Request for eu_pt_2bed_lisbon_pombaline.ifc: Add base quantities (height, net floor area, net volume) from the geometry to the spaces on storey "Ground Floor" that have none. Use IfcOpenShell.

First a look at what the model holds.

```python
import ifcopenshell
import ifcopenshell.util.element
import ifcopenshell.util.unit

model = ifcopenshell.open("eu_pt_2bed_lisbon_pombaline.ifc")
print(model.schema)
for unit_type in ("LENGTHUNIT", "AREAUNIT", "VOLUMEUNIT"):
    print(unit_type, ifcopenshell.util.unit.calculate_unit_scale(model, unit_type))
storey = next(s for s in model.by_type("IfcBuildingStorey") if s.Name == "Ground Floor")
spaces = [e for e in ifcopenshell.util.element.get_decomposition(storey) if e.is_a("IfcSpace")]
for e in sorted(spaces, key=lambda e: e.id()):
    print(e.id(), e.is_a(), e.Name, list(ifcopenshell.util.element.get_psets(e, qtos_only=True)), sep=" | ")
```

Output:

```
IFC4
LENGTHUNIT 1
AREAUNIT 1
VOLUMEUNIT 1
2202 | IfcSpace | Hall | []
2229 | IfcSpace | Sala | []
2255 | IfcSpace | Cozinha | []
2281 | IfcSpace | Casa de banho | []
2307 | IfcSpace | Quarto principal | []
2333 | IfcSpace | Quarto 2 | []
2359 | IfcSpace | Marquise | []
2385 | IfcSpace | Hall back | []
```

```python
import ifcopenshell
import ifcopenshell.api.pset
import ifcopenshell.geom
import ifcopenshell.util.element
import ifcopenshell.util.shape
import ifcopenshell.util.unit

model = ifcopenshell.open("eu_pt_2bed_lisbon_pombaline.ifc")
unit_scale = ifcopenshell.util.unit.calculate_unit_scale(model)
area_scale = ifcopenshell.util.unit.calculate_unit_scale(model, "AREAUNIT")
volume_scale = ifcopenshell.util.unit.calculate_unit_scale(model, "VOLUMEUNIT")
settings = ifcopenshell.geom.settings()

storey = next(s for s in model.by_type("IfcBuildingStorey") if s.Name == "Ground Floor")
spaces = [e for e in ifcopenshell.util.element.get_decomposition(storey) if e.is_a("IfcSpace")]

for e in sorted(spaces, key=lambda e: e.id()):
    if ifcopenshell.util.element.get_psets(e, qtos_only=True, should_inherit=False):
        continue
    # Geometry comes back in metres, in the element's own axes.
    shape = ifcopenshell.geom.create_shape(settings, e)
    values = {
        "Height": ifcopenshell.util.shape.get_z(shape.geometry) / unit_scale,
        "NetFloorArea": ifcopenshell.util.shape.get_footprint_area(shape.geometry) / area_scale,
        "NetVolume": ifcopenshell.util.shape.get_volume(shape.geometry) / volume_scale,
    }
    qto = ifcopenshell.api.pset.add_qto(model, product=e, name="Qto_SpaceBaseQuantities")
    ifcopenshell.api.pset.edit_qto(model, qto=qto, properties=values)
    print(e.id(), {k: round(v, 3) for k, v in values.items()})

model.write("eu_pt_2bed_lisbon_pombaline_rev.ifc")
```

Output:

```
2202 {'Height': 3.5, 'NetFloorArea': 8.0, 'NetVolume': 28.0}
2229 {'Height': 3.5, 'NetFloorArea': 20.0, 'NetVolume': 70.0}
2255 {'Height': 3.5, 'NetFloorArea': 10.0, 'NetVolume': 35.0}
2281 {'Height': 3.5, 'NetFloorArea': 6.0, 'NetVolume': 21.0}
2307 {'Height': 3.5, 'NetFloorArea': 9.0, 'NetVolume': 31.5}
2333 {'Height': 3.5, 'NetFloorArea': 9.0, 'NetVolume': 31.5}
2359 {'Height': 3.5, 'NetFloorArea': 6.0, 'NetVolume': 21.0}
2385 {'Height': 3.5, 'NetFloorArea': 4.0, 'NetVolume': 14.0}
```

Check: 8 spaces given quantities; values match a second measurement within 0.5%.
